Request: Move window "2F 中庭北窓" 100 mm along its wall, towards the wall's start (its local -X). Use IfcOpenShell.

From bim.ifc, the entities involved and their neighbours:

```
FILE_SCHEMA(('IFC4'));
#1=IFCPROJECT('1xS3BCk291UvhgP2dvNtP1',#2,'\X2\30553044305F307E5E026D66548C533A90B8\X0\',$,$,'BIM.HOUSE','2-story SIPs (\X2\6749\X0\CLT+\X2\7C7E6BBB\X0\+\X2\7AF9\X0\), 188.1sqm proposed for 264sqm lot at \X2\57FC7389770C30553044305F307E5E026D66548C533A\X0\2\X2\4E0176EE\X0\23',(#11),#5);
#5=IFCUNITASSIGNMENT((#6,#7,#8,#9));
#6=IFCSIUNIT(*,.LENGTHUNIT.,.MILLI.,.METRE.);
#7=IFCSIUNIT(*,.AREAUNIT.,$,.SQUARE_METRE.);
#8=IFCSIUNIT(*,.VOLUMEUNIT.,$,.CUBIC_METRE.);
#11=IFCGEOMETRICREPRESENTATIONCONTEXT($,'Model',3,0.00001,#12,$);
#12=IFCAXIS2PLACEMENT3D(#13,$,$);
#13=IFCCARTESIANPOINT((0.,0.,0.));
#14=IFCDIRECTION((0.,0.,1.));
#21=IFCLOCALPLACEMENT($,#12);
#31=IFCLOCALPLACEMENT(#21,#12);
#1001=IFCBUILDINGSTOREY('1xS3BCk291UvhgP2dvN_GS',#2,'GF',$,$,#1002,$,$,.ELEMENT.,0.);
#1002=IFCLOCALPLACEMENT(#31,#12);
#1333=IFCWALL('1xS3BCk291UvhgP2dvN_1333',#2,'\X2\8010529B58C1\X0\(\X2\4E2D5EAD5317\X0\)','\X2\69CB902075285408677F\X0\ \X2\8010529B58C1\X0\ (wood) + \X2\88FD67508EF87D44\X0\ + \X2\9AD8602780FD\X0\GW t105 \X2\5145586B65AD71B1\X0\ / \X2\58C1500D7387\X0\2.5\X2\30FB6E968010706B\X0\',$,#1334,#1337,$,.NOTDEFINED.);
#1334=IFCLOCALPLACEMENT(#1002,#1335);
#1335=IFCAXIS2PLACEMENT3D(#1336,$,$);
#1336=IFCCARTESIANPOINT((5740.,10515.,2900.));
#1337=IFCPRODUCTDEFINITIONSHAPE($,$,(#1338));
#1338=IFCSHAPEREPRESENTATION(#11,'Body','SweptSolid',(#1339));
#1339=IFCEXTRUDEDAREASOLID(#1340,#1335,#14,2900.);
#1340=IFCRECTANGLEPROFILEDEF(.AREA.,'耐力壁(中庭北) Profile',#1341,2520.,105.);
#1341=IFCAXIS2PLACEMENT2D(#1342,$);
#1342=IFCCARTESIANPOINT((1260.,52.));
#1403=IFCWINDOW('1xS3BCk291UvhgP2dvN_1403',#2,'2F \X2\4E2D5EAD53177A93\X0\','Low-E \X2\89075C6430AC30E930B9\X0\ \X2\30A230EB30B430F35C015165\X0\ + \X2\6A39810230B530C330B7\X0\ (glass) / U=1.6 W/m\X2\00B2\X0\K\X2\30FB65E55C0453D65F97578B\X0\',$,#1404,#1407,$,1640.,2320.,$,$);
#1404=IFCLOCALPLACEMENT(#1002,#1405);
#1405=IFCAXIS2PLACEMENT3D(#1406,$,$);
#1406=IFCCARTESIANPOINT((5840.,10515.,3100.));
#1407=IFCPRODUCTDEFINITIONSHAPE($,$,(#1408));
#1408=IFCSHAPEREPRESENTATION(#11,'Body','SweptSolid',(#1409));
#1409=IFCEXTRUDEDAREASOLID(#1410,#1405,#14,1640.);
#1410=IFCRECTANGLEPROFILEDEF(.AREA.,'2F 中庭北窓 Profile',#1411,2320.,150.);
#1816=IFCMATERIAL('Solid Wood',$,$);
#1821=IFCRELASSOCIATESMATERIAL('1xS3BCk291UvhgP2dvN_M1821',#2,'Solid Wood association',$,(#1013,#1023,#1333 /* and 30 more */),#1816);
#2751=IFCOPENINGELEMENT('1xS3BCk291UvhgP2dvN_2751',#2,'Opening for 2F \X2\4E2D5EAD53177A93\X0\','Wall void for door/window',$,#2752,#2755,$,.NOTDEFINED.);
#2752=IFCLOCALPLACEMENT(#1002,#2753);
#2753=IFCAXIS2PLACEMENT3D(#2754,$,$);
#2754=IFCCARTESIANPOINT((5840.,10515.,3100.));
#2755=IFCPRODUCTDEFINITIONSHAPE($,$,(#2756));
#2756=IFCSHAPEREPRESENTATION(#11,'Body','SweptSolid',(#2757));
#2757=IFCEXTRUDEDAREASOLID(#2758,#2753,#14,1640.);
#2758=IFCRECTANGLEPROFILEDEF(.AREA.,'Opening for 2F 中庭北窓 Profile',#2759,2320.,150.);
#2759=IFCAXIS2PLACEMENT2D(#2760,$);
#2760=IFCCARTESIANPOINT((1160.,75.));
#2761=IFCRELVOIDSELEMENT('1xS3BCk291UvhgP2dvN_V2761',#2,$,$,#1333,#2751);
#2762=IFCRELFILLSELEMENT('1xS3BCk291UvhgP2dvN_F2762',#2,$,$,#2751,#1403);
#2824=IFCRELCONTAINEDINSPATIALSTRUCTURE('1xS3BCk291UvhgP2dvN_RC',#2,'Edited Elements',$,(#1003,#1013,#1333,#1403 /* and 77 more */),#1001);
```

```python
import ifcopenshell
import ifcopenshell.api.geometry
import ifcopenshell.util.placement
import ifcopenshell.util.unit

model = ifcopenshell.open("bim.ifc")
unit_scale = ifcopenshell.util.unit.calculate_unit_scale(model)

window = model.by_guid("1xS3BCk291UvhgP2dvN_1403")
opening = window.FillsVoids[0].RelatingOpeningElement
wall = opening.VoidsElements[0].RelatingBuildingElement

wall_matrix = ifcopenshell.util.placement.get_local_placement(wall.ObjectPlacement)
shift = wall_matrix[:3, 0] * -0.1 / unit_scale
before = ifcopenshell.util.placement.get_local_placement(window.ObjectPlacement)[:3, 3].copy()

# The window is not placed relative to its opening, so move both.
for product in (opening, window):
    matrix = ifcopenshell.util.placement.get_local_placement(product.ObjectPlacement)
    matrix[:3, 3] += shift
    ifcopenshell.api.geometry.edit_object_placement(model, product=product, matrix=matrix, is_si=False)

after = ifcopenshell.util.placement.get_local_placement(window.ObjectPlacement)[:3, 3]
print("window moved by", (after - before).round(3) + 0.0)

model.write("bim-out.ifc")
```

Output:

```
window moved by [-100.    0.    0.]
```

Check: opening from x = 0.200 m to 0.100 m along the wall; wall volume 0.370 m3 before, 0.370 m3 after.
